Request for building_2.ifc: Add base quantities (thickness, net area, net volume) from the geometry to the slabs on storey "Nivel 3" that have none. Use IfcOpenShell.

First a look at what the model holds.

```python
import ifcopenshell
import ifcopenshell.util.element
import ifcopenshell.util.unit

model = ifcopenshell.open("building_2.ifc")
print(model.schema)
for unit_type in ("LENGTHUNIT", "AREAUNIT", "VOLUMEUNIT"):
    print(unit_type, ifcopenshell.util.unit.calculate_unit_scale(model, unit_type))
storey = next(s for s in model.by_type("IfcBuildingStorey") if s.Name == "Nivel 3")
slabs = [e for e in ifcopenshell.util.element.get_decomposition(storey) if e.is_a("IfcSlab")]
for e in sorted(slabs, key=lambda e: e.id()):
    print(e.id(), e.is_a(), e.Name, list(ifcopenshell.util.element.get_psets(e, qtos_only=True)), sep=" | ")
```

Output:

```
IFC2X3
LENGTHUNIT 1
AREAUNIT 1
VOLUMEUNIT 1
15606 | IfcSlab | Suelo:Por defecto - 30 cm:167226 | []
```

```python
import ifcopenshell
import ifcopenshell.api.pset
import ifcopenshell.geom
import ifcopenshell.util.element
import ifcopenshell.util.shape
import ifcopenshell.util.unit

model = ifcopenshell.open("building_2.ifc")
unit_scale = ifcopenshell.util.unit.calculate_unit_scale(model)
area_scale = ifcopenshell.util.unit.calculate_unit_scale(model, "AREAUNIT")
volume_scale = ifcopenshell.util.unit.calculate_unit_scale(model, "VOLUMEUNIT")
settings = ifcopenshell.geom.settings()

storey = next(s for s in model.by_type("IfcBuildingStorey") if s.Name == "Nivel 3")
slabs = [e for e in ifcopenshell.util.element.get_decomposition(storey) if e.is_a("IfcSlab")]

for e in sorted(slabs, key=lambda e: e.id()):
    if ifcopenshell.util.element.get_psets(e, qtos_only=True, should_inherit=False):
        continue
    # Geometry comes back in metres, in the element's own axes.
    shape = ifcopenshell.geom.create_shape(settings, e)
    values = {
        "Width": ifcopenshell.util.shape.get_z(shape.geometry) / unit_scale,
        "NetArea": ifcopenshell.util.shape.get_footprint_area(shape.geometry) / area_scale,
        "NetVolume": ifcopenshell.util.shape.get_volume(shape.geometry) / volume_scale,
    }
    qto = ifcopenshell.api.pset.add_qto(model, product=e, name="BaseQuantities")
    ifcopenshell.api.pset.edit_qto(model, qto=qto, properties=values)
    print(e.id(), {k: round(v, 3) for k, v in values.items()})

model.write("building_2_edited.ifc")
```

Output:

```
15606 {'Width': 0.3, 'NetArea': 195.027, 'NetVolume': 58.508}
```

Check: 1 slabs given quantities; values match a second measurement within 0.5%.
